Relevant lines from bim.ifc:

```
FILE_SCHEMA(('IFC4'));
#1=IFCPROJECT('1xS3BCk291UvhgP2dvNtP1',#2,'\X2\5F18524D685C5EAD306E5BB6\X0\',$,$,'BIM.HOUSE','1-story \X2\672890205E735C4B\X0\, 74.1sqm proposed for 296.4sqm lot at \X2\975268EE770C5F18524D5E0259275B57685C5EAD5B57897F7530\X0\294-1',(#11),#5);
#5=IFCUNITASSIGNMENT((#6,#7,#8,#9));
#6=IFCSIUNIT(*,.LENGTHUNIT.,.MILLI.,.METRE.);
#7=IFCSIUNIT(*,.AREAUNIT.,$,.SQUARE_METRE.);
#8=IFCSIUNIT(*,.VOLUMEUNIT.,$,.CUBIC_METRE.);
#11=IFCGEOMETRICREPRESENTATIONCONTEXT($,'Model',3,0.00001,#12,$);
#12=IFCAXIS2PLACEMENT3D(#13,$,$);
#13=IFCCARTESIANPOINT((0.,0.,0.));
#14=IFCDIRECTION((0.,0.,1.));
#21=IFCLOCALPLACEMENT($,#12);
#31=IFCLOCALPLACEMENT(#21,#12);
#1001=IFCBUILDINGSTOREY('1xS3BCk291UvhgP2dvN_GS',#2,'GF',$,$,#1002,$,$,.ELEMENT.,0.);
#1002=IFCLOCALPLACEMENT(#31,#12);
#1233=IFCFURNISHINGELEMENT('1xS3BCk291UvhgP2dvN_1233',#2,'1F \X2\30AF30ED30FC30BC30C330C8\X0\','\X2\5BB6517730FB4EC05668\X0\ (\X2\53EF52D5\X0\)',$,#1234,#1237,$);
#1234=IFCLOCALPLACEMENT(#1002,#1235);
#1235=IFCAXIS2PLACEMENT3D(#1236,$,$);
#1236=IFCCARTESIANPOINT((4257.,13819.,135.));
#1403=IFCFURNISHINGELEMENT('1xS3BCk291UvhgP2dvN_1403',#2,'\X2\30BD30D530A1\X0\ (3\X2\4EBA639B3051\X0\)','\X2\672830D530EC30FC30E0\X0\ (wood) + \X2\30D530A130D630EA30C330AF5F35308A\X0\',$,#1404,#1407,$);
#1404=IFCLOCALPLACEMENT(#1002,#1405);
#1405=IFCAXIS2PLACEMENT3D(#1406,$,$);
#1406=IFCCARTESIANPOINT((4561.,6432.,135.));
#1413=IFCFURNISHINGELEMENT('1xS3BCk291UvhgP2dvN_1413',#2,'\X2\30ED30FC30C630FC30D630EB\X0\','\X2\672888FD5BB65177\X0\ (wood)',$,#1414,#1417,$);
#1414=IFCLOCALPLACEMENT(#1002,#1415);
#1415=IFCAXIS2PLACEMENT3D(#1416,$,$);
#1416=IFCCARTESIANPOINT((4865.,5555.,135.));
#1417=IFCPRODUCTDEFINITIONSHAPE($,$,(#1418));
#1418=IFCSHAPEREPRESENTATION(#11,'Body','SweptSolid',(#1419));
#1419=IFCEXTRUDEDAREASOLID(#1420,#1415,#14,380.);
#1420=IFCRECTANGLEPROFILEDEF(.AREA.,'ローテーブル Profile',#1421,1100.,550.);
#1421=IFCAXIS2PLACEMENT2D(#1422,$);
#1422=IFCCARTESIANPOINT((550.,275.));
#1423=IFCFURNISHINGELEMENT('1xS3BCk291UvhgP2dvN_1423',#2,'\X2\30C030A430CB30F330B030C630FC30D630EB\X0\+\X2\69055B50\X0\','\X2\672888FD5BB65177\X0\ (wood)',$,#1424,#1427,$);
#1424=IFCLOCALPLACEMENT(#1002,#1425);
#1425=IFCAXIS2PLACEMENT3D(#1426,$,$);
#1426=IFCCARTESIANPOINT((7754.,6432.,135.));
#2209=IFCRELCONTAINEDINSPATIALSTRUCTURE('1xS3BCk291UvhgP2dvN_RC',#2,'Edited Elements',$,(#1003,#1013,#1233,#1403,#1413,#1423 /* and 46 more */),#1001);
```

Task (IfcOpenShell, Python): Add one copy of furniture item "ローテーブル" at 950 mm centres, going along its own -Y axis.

```python
import ifcopenshell
import ifcopenshell.api.geometry
import ifcopenshell.api.root
import ifcopenshell.util.element
import ifcopenshell.util.placement
import ifcopenshell.util.unit

model = ifcopenshell.open("bim.ifc")
unit_scale = ifcopenshell.util.unit.calculate_unit_scale(model)


def reuse_history(source, copy):
    """copy_class also copies each property set's owner history, people and application; keep the originals."""
    for rel in copy.IsDefinedBy:
        if rel.is_a("IfcRelDefinesByProperties") and (history := rel.RelatingPropertyDefinition.OwnerHistory):
            rel.RelatingPropertyDefinition.OwnerHistory = source.OwnerHistory
            ifcopenshell.util.element.remove_deep2(model, history)


source = model.by_guid("1xS3BCk291UvhgP2dvN_1413")
base = ifcopenshell.util.placement.get_local_placement(source.ObjectPlacement)
step = -base[:3, 1] * 0.95 / unit_scale

for i in range(1, 2):
    copy = ifcopenshell.api.root.copy_class(model, product=source)
    copy.Representation = ifcopenshell.util.element.copy_deep(
        model, source.Representation, exclude=["IfcGeometricRepresentationContext", "IfcRepresentationMap"]
    )
    reuse_history(source, copy)
    matrix = base.copy()
    matrix[:3, 3] += i * step
    print("added at", matrix[:3, 3].round(3) + 0.0)
    ifcopenshell.api.geometry.edit_object_placement(model, product=copy, matrix=matrix, is_si=False)

model.write("bim-out.ifc")
```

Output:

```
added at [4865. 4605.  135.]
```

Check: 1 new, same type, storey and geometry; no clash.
